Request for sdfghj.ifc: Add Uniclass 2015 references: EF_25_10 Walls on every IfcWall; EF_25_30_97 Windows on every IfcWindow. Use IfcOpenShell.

First a look at what the model holds.

```python
import ifcopenshell

model = ifcopenshell.open("sdfghj.ifc")
print(model.schema)
print("classifications:", [c.Name for c in model.by_type("IfcClassification")])
for ifc_class in ("IfcDoor", "IfcRoof", "IfcStair", "IfcWall", "IfcWindow"):
    print(ifc_class, len(model.by_type(ifc_class)))
```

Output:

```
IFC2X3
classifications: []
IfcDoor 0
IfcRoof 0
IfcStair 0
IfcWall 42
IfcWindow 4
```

```python
import ifcopenshell
import ifcopenshell.api.classification

model = ifcopenshell.open("sdfghj.ifc")

# IFC2X3 requires Source and Edition and has no link from the project to the system.
system = model.create_entity("IfcClassification", Source="NBS", Edition="2015", Name="Uniclass 2015")

codes = {
    "IfcWall": ("EF_25_10", "Walls"),
    "IfcWindow": ("EF_25_30_97", "Windows"),
}
for ifc_class, (code, name) in codes.items():
    products = model.by_type(ifc_class)
    ifcopenshell.api.classification.add_reference(
        model, products=products, classification=system, identification=code, name=name
    )
    print(code, len(products))

model.write("sdfghj_edited.ifc")
```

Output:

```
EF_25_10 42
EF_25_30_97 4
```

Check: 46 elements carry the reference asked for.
